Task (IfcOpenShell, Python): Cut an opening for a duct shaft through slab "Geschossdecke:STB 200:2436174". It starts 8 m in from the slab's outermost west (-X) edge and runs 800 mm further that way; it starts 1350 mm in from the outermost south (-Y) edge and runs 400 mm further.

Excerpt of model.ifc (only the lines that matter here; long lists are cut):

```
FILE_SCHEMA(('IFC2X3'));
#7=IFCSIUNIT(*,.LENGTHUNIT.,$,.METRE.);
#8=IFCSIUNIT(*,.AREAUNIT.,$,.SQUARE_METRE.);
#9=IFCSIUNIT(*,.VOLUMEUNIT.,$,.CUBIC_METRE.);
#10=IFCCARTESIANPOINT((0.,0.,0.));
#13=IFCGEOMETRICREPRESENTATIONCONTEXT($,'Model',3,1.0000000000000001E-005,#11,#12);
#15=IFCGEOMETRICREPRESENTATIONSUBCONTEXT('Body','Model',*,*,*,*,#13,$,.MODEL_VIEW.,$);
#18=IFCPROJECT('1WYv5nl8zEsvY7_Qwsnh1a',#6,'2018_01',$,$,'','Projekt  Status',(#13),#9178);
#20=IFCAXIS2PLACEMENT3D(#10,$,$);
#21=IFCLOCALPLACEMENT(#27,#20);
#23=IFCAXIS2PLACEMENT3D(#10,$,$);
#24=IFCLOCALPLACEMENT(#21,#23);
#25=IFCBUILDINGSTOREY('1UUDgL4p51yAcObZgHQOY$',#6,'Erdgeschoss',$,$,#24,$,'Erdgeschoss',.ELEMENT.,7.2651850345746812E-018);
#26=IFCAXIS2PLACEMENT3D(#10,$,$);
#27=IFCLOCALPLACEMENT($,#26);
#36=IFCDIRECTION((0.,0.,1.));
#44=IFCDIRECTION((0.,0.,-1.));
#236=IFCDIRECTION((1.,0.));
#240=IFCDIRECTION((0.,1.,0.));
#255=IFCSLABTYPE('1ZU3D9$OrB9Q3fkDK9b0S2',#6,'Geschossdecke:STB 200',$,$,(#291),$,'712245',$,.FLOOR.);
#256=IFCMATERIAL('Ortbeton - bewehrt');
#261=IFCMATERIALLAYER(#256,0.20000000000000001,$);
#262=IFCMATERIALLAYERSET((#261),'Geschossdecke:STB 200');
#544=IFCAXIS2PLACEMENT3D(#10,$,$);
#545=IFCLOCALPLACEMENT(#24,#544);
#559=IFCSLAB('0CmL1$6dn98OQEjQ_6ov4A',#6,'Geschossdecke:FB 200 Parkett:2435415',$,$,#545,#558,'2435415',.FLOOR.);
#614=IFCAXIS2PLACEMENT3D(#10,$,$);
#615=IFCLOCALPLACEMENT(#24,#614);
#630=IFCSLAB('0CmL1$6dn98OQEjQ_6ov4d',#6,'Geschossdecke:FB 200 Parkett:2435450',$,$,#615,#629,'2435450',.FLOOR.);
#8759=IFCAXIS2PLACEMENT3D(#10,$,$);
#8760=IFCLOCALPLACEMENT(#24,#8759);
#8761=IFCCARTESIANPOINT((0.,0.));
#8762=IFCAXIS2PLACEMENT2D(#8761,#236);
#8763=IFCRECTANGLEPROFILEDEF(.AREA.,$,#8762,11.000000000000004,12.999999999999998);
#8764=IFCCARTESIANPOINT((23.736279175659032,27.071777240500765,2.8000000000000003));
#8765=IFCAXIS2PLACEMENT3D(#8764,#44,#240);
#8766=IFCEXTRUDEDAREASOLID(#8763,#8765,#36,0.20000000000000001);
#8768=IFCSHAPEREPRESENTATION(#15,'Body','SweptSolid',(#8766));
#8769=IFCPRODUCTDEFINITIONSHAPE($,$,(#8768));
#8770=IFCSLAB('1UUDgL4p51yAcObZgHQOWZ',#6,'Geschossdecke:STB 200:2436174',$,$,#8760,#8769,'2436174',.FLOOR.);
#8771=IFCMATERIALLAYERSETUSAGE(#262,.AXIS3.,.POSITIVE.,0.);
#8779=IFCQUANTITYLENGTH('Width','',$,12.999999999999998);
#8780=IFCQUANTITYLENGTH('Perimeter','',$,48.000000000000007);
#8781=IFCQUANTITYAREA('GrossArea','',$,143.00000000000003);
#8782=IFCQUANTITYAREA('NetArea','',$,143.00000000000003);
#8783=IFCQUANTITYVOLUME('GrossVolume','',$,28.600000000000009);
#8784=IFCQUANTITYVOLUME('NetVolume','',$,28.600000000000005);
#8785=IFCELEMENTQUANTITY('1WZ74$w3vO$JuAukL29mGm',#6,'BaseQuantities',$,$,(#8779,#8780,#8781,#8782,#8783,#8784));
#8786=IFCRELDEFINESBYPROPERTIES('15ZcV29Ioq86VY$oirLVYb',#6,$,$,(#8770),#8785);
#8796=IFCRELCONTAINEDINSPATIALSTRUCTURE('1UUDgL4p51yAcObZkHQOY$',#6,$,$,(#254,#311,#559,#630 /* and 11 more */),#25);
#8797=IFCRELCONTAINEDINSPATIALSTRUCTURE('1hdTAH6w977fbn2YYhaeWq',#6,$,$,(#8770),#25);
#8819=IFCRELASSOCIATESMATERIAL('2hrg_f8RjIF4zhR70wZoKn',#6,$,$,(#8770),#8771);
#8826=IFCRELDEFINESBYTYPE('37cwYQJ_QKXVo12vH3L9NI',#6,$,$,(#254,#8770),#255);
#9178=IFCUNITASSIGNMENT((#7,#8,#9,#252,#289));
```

```python
import numpy as np
import ifcopenshell
import ifcopenshell.api.feature
import ifcopenshell.api.geometry
import ifcopenshell.api.pset
import ifcopenshell.api.root
import ifcopenshell.geom
import ifcopenshell.util.element
import ifcopenshell.util.placement
import ifcopenshell.util.representation
import ifcopenshell.util.shape
import ifcopenshell.util.unit

model = ifcopenshell.open("model.ifc")
unit_scale = ifcopenshell.util.unit.calculate_unit_scale(model)
area_scale = ifcopenshell.util.unit.calculate_unit_scale(model, "AREAUNIT")
volume_scale = ifcopenshell.util.unit.calculate_unit_scale(model, "VOLUMEUNIT")
settings = ifcopenshell.geom.settings()


def volume(element):
    """Net volume in cubic metres, openings subtracted."""
    shape = ifcopenshell.geom.create_shape(settings, element)
    return ifcopenshell.util.shape.get_volume(shape.geometry)


slab = model.by_guid("1UUDgL4p51yAcObZgHQOWZ")
before = volume(slab)

# Extent in the slab's own axes, in metres. The edges named are its -X and -Y sides.
slab_shape = ifcopenshell.geom.create_shape(settings, slab)
vertices = ifcopenshell.util.shape.get_vertices(slab_shape.geometry)
x_min, y_min, bottom = vertices.min(axis=0)
top = vertices[:, 2].max()

opening = ifcopenshell.api.root.create_entity(model, ifc_class="IfcOpeningElement", name="Duct shaft opening")
context = ifcopenshell.util.representation.get_context(model, "Model", "Body", "MODEL_VIEW")
width, depth = 0.8, 0.4
outline = [(0.0, 0.0), (width, 0.0), (width, depth), (0.0, depth), (0.0, 0.0)]
# Overshoot both faces by 50 mm so the cut is clean.
shape = ifcopenshell.api.geometry.add_slab_representation(
    model, context=context, depth=top - bottom + 0.1, polyline=outline
)
ifcopenshell.api.geometry.assign_representation(model, product=opening, representation=shape)

matrix = ifcopenshell.util.placement.get_local_placement(slab.ObjectPlacement)
matrix[:, 3] = matrix @ np.append(np.array([x_min + 8, y_min + 1.35, bottom - 0.05]) / unit_scale, 1.0)
ifcopenshell.api.geometry.edit_object_placement(model, product=opening, matrix=matrix, is_si=False)
ifcopenshell.api.feature.add_feature(model, feature=opening, element=slab)

after = volume(slab)

# Update the slab's stored quantities.
qto = model.by_id(ifcopenshell.util.element.get_pset(slab, "BaseQuantities", should_inherit=False)["id"])
ifcopenshell.api.pset.edit_qto(model, qto=qto, properties={
    "NetArea": after / (top - bottom) / area_scale,
    "NetVolume": after / volume_scale,
})

print(f"slab volume {before:.3f} -> {after:.3f} m3")

model.write("model_updated.ifc")
```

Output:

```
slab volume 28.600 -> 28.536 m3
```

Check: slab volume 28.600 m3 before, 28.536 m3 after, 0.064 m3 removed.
